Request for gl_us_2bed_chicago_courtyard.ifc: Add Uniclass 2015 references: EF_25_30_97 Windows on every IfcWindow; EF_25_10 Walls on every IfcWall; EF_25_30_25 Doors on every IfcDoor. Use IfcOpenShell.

First a look at what the model holds.

```python
import ifcopenshell

model = ifcopenshell.open("gl_us_2bed_chicago_courtyard.ifc")
print(model.schema)
print("classifications:", [c.Name for c in model.by_type("IfcClassification")])
for ifc_class in ("IfcDoor", "IfcRoof", "IfcStair", "IfcWall", "IfcWindow"):
    print(ifc_class, len(model.by_type(ifc_class)))
```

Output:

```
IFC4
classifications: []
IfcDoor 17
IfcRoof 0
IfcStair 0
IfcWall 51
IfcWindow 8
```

```python
import ifcopenshell
import ifcopenshell.api.classification

model = ifcopenshell.open("gl_us_2bed_chicago_courtyard.ifc")

system = ifcopenshell.api.classification.add_classification(model, classification="Uniclass 2015")

codes = {
    "IfcWindow": ("EF_25_30_97", "Windows"),
    "IfcWall": ("EF_25_10", "Walls"),
    "IfcDoor": ("EF_25_30_25", "Doors"),
}
for ifc_class, (code, name) in codes.items():
    products = model.by_type(ifc_class)
    ifcopenshell.api.classification.add_reference(
        model, products=products, classification=system, identification=code, name=name
    )
    print(code, len(products))

model.write("gl_us_2bed_chicago_courtyard_updated.ifc")
```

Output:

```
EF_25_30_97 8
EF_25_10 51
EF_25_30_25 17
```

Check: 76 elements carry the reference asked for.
